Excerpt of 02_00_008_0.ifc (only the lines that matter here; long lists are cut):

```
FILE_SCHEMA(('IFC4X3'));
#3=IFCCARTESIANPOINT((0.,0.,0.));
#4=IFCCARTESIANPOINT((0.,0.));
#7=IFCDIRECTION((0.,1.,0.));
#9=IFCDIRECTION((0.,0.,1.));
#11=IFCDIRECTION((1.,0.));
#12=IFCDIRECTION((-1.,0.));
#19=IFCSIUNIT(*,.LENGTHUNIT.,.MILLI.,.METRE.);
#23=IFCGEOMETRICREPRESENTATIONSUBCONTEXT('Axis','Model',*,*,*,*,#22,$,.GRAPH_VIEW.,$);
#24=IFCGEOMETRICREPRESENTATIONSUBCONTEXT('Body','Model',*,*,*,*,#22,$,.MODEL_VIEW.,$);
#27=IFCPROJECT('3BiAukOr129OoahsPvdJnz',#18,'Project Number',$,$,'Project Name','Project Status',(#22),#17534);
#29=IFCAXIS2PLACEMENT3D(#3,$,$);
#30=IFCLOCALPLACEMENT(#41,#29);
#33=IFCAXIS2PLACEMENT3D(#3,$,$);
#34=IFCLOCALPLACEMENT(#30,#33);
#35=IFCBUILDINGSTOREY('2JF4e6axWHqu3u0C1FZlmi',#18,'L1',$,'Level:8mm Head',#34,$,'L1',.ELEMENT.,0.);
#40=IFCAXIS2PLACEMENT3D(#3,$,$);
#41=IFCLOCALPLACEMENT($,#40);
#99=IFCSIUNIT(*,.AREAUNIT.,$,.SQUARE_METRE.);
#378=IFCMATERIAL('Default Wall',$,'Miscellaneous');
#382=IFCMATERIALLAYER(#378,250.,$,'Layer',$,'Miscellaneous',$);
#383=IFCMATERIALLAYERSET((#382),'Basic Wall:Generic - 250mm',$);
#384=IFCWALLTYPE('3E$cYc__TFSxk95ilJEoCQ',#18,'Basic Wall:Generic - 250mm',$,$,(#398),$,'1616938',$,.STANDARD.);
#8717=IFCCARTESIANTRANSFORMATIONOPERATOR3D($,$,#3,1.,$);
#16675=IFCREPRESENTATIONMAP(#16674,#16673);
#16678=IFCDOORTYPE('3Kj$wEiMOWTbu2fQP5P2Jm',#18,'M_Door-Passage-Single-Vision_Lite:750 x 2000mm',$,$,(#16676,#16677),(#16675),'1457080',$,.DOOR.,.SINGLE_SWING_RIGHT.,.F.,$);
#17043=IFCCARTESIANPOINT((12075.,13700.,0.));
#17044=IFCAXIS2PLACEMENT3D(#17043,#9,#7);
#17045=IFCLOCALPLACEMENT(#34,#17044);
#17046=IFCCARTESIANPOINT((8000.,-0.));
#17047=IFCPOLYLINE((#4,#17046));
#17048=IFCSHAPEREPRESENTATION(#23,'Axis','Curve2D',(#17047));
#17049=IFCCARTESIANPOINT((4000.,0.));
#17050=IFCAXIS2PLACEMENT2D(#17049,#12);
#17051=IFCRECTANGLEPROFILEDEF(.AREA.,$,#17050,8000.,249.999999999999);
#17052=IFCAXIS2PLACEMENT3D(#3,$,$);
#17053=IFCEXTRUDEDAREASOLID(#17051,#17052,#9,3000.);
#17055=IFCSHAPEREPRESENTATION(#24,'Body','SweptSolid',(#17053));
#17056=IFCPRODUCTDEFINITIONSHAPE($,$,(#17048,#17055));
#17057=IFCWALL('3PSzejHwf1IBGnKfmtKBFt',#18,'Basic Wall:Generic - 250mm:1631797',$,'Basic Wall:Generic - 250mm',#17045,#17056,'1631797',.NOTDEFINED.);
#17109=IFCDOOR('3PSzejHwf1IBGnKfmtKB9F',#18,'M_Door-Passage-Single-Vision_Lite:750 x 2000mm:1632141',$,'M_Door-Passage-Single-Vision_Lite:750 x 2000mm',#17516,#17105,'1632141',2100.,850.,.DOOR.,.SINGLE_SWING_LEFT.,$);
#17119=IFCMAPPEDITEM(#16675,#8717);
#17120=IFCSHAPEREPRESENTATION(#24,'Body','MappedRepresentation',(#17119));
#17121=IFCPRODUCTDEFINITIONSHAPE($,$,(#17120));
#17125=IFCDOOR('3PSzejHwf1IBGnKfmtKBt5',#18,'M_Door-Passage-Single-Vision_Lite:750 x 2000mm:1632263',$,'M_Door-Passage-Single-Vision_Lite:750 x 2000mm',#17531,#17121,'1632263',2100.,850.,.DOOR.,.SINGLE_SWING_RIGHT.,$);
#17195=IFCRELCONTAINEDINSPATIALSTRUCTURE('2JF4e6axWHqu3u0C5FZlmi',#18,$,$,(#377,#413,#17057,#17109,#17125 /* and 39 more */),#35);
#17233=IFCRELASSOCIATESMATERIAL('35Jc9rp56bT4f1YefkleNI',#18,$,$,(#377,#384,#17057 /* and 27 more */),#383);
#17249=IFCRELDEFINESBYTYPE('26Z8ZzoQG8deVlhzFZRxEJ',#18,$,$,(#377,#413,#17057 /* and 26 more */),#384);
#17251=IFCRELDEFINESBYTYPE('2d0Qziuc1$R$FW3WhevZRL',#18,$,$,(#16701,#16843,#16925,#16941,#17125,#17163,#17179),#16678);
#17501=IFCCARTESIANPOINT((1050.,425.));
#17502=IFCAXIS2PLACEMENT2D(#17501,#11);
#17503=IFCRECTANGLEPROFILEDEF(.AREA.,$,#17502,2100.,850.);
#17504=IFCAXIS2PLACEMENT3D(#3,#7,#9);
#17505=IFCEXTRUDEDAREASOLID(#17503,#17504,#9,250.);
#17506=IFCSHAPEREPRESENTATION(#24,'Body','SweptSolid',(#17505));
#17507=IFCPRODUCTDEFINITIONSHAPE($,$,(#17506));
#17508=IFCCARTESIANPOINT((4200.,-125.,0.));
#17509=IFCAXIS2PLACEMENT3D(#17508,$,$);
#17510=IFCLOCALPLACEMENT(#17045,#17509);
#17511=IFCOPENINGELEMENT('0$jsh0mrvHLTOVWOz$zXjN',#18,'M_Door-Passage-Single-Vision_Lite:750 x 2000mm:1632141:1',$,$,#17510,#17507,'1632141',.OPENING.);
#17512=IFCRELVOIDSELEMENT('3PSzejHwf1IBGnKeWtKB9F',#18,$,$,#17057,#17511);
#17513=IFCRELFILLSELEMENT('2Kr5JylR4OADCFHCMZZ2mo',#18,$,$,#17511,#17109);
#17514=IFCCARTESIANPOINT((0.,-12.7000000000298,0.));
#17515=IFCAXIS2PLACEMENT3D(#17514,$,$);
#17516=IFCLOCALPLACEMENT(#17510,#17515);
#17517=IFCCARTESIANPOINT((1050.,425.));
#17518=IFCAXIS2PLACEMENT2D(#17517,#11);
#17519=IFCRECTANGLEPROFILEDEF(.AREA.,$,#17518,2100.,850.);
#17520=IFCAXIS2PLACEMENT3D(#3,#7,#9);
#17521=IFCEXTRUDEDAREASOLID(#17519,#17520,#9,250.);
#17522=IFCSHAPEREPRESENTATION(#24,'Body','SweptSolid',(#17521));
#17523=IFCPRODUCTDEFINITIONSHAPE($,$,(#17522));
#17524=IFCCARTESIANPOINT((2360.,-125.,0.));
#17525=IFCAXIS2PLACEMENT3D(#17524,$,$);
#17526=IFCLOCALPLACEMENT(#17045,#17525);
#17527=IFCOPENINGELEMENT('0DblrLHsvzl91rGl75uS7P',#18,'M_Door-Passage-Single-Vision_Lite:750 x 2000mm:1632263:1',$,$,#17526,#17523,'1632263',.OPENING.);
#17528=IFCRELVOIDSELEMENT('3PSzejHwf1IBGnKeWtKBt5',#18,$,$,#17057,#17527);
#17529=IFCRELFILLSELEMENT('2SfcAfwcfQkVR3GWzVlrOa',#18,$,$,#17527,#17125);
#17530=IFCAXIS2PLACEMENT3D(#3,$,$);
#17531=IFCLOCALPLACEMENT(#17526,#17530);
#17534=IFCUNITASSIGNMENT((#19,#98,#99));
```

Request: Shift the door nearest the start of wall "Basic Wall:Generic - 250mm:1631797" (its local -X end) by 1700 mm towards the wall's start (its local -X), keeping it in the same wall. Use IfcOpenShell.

```python
import ifcopenshell
import ifcopenshell.api.geometry
import ifcopenshell.util.placement

model = ifcopenshell.open("02_00_008_0.ifc")

door = model.by_guid("3PSzejHwf1IBGnKfmtKBt5")
opening = door.FillsVoids[0].RelatingOpeningElement
wall = opening.VoidsElements[0].RelatingBuildingElement

wall_matrix = ifcopenshell.util.placement.get_local_placement(wall.ObjectPlacement)
shift = wall_matrix[:3, 0] * -1700.0
before = ifcopenshell.util.placement.get_local_placement(door.ObjectPlacement)[:3, 3].copy()

# The door is placed relative to its opening, so it follows when the opening moves.
matrix = ifcopenshell.util.placement.get_local_placement(opening.ObjectPlacement)
matrix[:3, 3] += shift
ifcopenshell.api.geometry.edit_object_placement(
    model, product=opening, matrix=matrix, is_si=False, should_transform_children=True
)

after = ifcopenshell.util.placement.get_local_placement(door.ObjectPlacement)[:3, 3]
print("door moved by", (after - before).round(3) + 0.0)

model.write("02_00_008_0_updated.ifc")
```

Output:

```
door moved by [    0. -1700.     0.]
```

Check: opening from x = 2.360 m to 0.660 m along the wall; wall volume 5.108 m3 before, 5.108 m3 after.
